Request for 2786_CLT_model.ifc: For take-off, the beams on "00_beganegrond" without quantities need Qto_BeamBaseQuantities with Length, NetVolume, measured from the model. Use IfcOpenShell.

First a look at what the model holds.

```python
import ifcopenshell
import ifcopenshell.util.element
import ifcopenshell.util.unit

model = ifcopenshell.open("2786_CLT_model.ifc")
print(model.schema)
for unit_type in ("LENGTHUNIT", "AREAUNIT", "VOLUMEUNIT"):
    print(unit_type, ifcopenshell.util.unit.calculate_unit_scale(model, unit_type))
storey = next(s for s in model.by_type("IfcBuildingStorey") if s.Name == "00_beganegrond")
beams = [e for e in ifcopenshell.util.element.get_decomposition(storey) if e.is_a("IfcBeam")]
for e in sorted(beams, key=lambda e: e.id()):
    print(e.id(), e.is_a(), e.Name, list(ifcopenshell.util.element.get_psets(e, qtos_only=True)), sep=" | ")
```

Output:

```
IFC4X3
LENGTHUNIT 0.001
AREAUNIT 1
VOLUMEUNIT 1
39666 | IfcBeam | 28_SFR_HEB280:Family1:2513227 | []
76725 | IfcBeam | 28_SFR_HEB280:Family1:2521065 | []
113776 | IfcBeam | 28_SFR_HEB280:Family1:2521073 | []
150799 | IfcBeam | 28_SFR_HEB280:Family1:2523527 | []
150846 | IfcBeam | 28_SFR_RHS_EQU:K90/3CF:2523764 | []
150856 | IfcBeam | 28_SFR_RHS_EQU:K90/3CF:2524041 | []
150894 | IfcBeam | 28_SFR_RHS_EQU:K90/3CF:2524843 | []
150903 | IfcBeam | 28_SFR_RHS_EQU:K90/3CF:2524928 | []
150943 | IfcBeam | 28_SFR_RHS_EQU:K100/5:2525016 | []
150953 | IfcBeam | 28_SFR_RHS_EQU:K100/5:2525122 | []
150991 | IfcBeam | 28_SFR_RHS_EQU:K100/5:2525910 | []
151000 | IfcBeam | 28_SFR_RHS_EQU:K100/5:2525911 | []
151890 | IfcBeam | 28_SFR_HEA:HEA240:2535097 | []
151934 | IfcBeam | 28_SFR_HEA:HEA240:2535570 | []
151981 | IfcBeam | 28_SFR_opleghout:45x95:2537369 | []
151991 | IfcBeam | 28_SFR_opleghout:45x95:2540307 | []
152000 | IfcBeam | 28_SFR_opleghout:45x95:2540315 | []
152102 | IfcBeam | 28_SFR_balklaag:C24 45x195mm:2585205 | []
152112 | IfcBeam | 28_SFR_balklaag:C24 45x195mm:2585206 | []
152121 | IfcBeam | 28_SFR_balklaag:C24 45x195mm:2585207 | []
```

```python
import ifcopenshell
import ifcopenshell.api.pset
import ifcopenshell.geom
import ifcopenshell.util.element
import ifcopenshell.util.shape
import ifcopenshell.util.unit

model = ifcopenshell.open("2786_CLT_model.ifc")
unit_scale = ifcopenshell.util.unit.calculate_unit_scale(model)
volume_scale = ifcopenshell.util.unit.calculate_unit_scale(model, "VOLUMEUNIT")
settings = ifcopenshell.geom.settings()

storey = next(s for s in model.by_type("IfcBuildingStorey") if s.Name == "00_beganegrond")
beams = [e for e in ifcopenshell.util.element.get_decomposition(storey) if e.is_a("IfcBeam")]

for e in sorted(beams, key=lambda e: e.id()):
    if ifcopenshell.util.element.get_psets(e, qtos_only=True, should_inherit=False):
        continue
    # Geometry comes back in metres, in the element's own axes.
    shape = ifcopenshell.geom.create_shape(settings, e)
    values = {
        "Length": ifcopenshell.util.shape.get_max_xyz(shape.geometry) / unit_scale,
        "NetVolume": ifcopenshell.util.shape.get_volume(shape.geometry) / volume_scale,
    }
    qto = ifcopenshell.api.pset.add_qto(model, product=e, name="Qto_BeamBaseQuantities")
    ifcopenshell.api.pset.edit_qto(model, qto=qto, properties=values)
    print(e.id(), {k: round(v, 3) for k, v in values.items()})

model.write("2786_CLT_model_edited.ifc")
```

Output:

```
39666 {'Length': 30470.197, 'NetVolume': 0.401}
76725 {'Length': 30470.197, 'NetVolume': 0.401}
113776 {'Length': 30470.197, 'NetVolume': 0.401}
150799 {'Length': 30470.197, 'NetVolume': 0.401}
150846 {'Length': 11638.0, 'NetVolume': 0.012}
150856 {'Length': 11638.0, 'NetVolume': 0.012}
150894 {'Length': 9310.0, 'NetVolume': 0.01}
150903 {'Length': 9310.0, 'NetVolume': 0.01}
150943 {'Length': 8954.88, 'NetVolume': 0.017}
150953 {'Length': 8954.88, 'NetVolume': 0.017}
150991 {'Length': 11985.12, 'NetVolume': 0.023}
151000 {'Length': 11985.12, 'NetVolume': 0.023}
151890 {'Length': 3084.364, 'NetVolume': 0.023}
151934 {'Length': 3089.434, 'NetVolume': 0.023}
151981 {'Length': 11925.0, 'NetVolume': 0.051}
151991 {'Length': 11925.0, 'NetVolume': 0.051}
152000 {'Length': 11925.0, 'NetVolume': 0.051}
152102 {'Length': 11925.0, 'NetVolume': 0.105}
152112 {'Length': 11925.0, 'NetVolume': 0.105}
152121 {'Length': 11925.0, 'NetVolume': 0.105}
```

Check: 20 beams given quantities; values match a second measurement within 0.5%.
